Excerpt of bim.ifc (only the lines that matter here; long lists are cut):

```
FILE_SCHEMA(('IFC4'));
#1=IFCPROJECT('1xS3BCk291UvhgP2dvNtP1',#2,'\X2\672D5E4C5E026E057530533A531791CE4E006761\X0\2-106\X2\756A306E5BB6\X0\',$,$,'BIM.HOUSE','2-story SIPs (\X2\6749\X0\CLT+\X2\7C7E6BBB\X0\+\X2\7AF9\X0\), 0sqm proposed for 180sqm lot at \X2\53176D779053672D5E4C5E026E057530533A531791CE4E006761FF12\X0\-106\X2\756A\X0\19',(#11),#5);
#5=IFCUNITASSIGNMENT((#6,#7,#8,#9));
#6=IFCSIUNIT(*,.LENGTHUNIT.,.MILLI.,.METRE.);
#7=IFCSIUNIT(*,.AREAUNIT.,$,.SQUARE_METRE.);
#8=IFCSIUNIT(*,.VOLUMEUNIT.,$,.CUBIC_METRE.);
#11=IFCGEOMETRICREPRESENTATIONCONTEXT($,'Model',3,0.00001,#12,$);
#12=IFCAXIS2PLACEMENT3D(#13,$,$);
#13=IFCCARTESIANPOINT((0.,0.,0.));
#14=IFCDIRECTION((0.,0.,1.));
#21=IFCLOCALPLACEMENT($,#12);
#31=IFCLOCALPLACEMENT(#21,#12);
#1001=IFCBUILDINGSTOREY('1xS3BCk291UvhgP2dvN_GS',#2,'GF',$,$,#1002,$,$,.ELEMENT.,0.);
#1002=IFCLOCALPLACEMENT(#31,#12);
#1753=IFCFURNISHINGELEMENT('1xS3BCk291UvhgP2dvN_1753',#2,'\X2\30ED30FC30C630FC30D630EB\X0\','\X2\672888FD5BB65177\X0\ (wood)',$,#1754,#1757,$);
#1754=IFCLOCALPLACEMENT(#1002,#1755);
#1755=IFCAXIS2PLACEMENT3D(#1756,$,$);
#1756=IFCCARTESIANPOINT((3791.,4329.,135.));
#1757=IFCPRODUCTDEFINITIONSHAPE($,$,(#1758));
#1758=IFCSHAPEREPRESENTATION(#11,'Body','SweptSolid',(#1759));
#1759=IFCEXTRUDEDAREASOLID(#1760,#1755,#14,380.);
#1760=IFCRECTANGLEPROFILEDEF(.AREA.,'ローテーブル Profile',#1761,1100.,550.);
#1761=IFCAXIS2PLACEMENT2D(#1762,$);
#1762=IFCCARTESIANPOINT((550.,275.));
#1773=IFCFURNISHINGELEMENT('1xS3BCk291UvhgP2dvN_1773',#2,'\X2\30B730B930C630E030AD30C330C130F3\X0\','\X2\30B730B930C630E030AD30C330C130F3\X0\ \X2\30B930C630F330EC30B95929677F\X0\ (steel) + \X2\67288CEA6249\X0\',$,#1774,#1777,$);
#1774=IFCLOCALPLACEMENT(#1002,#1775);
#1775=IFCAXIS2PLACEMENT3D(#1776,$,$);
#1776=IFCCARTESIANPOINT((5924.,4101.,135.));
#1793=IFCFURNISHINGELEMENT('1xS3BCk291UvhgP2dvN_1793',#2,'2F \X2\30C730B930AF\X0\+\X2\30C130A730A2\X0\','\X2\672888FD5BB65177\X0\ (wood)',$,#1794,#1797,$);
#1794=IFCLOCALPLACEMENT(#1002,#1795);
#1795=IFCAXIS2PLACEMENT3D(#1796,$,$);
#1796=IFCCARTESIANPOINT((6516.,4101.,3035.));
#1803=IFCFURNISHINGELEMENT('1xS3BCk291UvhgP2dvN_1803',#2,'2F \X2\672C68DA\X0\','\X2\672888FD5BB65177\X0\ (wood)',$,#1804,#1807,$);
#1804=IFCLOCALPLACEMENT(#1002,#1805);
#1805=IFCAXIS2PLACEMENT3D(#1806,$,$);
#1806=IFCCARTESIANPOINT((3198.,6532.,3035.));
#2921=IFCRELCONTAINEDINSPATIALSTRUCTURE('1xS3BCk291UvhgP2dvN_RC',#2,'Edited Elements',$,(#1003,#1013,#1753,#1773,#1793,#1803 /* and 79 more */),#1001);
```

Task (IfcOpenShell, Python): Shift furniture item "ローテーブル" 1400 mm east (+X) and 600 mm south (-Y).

```python
import ifcopenshell
import ifcopenshell.api.geometry
import ifcopenshell.util.placement

model = ifcopenshell.open("bim.ifc")

item = model.by_guid("1xS3BCk291UvhgP2dvN_1753")
matrix = ifcopenshell.util.placement.get_local_placement(item.ObjectPlacement)
matrix[0, 3] += 1400.0
matrix[1, 3] -= 600.0
ifcopenshell.api.geometry.edit_object_placement(model, product=item, matrix=matrix, is_si=False)

print(ifcopenshell.util.placement.get_local_placement(item.ObjectPlacement).round(3) + 0.0)

model.write("bim_edited.ifc")
```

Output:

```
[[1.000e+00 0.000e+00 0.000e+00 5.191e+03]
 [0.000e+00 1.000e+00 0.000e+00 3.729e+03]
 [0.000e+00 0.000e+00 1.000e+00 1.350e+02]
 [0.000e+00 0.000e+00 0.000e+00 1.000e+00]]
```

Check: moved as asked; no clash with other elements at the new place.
